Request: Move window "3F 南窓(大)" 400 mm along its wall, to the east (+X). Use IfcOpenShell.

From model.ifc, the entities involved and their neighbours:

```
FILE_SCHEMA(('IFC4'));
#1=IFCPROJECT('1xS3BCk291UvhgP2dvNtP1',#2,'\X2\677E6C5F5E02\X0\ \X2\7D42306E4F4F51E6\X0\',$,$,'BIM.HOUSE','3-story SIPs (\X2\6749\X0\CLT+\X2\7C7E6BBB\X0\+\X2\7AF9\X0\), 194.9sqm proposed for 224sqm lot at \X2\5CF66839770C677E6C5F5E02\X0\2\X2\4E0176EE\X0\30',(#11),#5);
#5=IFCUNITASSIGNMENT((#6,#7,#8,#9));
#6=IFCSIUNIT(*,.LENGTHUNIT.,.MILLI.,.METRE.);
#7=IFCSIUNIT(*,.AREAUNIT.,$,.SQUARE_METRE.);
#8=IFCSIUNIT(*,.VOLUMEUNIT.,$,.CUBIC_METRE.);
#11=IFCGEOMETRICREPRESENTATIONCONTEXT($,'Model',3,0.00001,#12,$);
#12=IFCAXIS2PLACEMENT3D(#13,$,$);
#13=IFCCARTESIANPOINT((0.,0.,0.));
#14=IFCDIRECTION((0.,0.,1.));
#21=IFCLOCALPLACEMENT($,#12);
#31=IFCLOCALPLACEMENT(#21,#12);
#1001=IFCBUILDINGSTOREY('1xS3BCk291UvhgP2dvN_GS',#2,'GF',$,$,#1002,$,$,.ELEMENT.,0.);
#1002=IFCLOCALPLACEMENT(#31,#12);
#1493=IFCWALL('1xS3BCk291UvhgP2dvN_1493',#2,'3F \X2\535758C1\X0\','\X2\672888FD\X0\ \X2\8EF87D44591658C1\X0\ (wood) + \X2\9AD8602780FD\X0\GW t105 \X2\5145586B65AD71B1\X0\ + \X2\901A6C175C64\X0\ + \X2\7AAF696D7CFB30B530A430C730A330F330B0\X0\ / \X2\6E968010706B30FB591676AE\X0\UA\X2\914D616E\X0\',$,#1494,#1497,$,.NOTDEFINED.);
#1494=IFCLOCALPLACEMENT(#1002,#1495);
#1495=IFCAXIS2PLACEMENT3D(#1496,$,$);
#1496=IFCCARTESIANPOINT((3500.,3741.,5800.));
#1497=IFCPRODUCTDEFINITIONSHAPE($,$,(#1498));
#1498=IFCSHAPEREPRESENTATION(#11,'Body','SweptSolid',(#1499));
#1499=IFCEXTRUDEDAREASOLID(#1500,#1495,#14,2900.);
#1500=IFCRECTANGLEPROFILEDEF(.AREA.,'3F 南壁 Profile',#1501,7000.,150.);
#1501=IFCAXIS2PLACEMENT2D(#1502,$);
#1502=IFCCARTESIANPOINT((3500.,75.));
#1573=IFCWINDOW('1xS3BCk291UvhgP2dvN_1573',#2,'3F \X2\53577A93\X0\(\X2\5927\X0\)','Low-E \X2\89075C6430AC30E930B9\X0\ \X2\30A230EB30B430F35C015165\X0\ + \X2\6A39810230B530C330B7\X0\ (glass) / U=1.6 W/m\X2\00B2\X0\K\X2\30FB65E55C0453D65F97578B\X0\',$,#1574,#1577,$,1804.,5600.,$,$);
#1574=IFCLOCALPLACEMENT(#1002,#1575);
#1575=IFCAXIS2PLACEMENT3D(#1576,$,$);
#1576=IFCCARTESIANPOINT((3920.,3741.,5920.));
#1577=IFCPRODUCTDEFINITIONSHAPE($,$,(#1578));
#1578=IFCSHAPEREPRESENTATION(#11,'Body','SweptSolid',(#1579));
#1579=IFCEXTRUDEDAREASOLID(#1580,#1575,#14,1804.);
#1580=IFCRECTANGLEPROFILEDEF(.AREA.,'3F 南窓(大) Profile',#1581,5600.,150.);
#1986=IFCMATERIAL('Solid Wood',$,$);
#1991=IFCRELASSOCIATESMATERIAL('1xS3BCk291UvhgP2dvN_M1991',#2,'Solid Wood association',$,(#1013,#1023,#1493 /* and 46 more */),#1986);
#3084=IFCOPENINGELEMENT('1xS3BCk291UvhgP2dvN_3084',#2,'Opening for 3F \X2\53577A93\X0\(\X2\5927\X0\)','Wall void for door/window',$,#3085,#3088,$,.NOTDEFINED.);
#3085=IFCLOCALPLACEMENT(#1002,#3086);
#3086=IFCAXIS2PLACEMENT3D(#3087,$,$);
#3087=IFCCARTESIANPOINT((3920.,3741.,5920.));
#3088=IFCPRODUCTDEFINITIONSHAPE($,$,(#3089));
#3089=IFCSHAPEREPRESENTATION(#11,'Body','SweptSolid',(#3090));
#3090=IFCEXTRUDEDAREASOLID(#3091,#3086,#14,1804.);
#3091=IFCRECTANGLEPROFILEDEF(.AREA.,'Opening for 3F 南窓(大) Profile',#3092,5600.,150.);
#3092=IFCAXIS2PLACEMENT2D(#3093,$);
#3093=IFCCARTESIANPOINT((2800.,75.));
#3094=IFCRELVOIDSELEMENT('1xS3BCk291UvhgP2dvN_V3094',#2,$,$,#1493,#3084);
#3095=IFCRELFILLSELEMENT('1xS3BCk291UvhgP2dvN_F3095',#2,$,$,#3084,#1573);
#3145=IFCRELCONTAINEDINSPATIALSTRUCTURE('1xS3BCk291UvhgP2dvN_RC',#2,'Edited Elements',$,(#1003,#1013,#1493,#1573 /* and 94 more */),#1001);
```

```python
import ifcopenshell
import ifcopenshell.api.geometry
import ifcopenshell.util.placement
import ifcopenshell.util.unit

model = ifcopenshell.open("model.ifc")
unit_scale = ifcopenshell.util.unit.calculate_unit_scale(model)

window = model.by_guid("1xS3BCk291UvhgP2dvN_1573")
opening = window.FillsVoids[0].RelatingOpeningElement
wall = opening.VoidsElements[0].RelatingBuildingElement

wall_matrix = ifcopenshell.util.placement.get_local_placement(wall.ObjectPlacement)
shift = wall_matrix[:3, 0] * 0.4 / unit_scale
before = ifcopenshell.util.placement.get_local_placement(window.ObjectPlacement)[:3, 3].copy()

# The window is not placed relative to its opening, so move both.
for product in (opening, window):
    matrix = ifcopenshell.util.placement.get_local_placement(product.ObjectPlacement)
    matrix[:3, 3] += shift
    ifcopenshell.api.geometry.edit_object_placement(model, product=product, matrix=matrix, is_si=False)

after = ifcopenshell.util.placement.get_local_placement(window.ObjectPlacement)[:3, 3]
print("window moved by", (after - before).round(3) + 0.0)

model.write("model_rev.ifc")
```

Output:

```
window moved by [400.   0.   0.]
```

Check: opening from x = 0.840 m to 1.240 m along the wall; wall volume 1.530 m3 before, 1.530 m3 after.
